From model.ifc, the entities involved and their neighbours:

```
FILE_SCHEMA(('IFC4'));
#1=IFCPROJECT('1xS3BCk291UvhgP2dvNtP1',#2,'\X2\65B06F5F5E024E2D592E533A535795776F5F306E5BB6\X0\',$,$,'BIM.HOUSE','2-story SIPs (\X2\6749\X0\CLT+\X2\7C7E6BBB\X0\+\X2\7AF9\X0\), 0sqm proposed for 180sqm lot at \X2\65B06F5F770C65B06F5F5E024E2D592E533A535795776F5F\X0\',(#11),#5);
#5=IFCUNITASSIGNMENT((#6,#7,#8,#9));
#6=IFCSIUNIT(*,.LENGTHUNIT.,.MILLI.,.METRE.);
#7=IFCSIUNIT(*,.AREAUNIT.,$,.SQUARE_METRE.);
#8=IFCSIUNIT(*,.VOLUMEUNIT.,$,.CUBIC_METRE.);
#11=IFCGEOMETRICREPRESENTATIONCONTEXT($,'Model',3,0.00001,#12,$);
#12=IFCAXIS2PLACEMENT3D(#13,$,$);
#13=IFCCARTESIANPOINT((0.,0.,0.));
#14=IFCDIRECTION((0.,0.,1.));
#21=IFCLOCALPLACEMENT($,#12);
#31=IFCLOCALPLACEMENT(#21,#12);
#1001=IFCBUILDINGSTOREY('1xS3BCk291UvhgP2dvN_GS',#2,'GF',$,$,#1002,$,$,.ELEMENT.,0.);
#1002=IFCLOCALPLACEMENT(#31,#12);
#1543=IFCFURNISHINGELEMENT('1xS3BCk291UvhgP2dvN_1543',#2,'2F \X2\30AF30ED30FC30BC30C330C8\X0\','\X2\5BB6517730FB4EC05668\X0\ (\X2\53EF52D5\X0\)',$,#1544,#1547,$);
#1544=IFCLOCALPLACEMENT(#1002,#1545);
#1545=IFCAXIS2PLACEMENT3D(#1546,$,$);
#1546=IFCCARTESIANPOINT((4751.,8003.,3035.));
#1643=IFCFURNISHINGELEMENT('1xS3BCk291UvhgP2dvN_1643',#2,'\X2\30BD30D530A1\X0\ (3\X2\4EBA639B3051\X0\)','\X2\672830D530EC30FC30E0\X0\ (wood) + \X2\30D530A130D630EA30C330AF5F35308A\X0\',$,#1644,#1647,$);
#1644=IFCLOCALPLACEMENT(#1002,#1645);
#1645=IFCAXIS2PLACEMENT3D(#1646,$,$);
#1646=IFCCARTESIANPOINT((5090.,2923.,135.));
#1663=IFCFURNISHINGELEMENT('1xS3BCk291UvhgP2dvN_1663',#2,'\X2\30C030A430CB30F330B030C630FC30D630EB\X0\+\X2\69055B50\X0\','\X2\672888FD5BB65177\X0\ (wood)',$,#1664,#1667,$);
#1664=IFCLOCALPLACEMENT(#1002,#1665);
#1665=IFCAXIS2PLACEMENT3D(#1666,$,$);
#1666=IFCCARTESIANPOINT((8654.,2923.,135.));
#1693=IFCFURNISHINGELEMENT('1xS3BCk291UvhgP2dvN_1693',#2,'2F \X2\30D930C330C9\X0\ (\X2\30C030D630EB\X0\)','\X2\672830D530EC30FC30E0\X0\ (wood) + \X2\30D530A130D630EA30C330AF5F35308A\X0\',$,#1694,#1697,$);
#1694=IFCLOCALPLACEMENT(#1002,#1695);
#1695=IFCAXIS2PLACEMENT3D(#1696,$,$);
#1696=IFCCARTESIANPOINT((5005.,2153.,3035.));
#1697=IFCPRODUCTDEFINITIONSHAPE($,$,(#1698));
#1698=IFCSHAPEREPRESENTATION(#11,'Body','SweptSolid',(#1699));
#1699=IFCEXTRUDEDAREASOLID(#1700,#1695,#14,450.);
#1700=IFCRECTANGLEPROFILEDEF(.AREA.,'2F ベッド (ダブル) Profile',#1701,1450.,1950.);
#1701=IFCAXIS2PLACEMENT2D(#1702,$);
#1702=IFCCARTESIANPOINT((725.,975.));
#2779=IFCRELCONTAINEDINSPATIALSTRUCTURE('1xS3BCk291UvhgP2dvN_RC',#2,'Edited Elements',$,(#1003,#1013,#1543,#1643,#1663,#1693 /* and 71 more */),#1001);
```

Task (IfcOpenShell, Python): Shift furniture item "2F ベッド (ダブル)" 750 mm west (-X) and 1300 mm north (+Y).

```python
import ifcopenshell
import ifcopenshell.api.geometry
import ifcopenshell.util.placement
import ifcopenshell.util.unit

model = ifcopenshell.open("model.ifc")
unit_scale = ifcopenshell.util.unit.calculate_unit_scale(model)

item = model.by_guid("1xS3BCk291UvhgP2dvN_1693")
matrix = ifcopenshell.util.placement.get_local_placement(item.ObjectPlacement)
matrix[0, 3] -= 0.75 / unit_scale
matrix[1, 3] += 1.3 / unit_scale
ifcopenshell.api.geometry.edit_object_placement(model, product=item, matrix=matrix, is_si=False)

print(ifcopenshell.util.placement.get_local_placement(item.ObjectPlacement).round(3) + 0.0)

model.write("model_edited.ifc")
```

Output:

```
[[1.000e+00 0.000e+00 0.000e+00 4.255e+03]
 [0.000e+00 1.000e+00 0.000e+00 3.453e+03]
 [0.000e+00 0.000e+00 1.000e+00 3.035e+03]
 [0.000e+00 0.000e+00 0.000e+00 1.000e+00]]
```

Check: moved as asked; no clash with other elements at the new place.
